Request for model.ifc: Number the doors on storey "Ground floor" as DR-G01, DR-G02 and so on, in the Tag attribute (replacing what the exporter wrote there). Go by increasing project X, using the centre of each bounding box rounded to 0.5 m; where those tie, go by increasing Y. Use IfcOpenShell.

First a look at what the model holds.

```python
import ifcopenshell
import ifcopenshell.util.element
import ifcopenshell.util.placement

model = ifcopenshell.open("model.ifc")
print(model.schema)
storey = next(s for s in model.by_type("IfcBuildingStorey") if s.Name == "Ground floor")
doors = [e for e in ifcopenshell.util.element.get_decomposition(storey) if e.is_a("IfcDoor")]
for e in sorted(doors, key=lambda e: e.id()):
    origin = ifcopenshell.util.placement.get_local_placement(e.ObjectPlacement)[:3, 3]
    print(e.id(), e.Tag, e.Name, origin.round(2) + 0.0, sep=" | ")
```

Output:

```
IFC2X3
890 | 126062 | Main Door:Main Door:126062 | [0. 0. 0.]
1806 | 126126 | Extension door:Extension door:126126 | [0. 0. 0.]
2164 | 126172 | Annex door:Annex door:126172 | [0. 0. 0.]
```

```python
import ifcopenshell
import ifcopenshell.geom
import ifcopenshell.util.element
import ifcopenshell.util.shape

model = ifcopenshell.open("model.ifc")
settings = ifcopenshell.geom.settings()
settings.set("use-world-coords", True)


def centre(element):
    shape = ifcopenshell.geom.create_shape(settings, element)
    return ifcopenshell.util.shape.get_bbox_centroid(shape.geometry)


storey = next(s for s in model.by_type("IfcBuildingStorey") if s.Name == "Ground floor")
doors = [e for e in ifcopenshell.util.element.get_decomposition(storey) if e.is_a("IfcDoor")]

# Insertion points can sit at a corner or the storey origin, so sort by the geometry (in metres).
centres = {e: centre(e) for e in doors}
doors.sort(key=lambda e: (round(centres[e][0] / 0.5), centres[e][1]))

for i, e in enumerate(doors, start=1):
    number = f"DR-G{i:02d}"
    e.Tag = number
    print(e.id(), number)

model.write("model_edited.ifc")
```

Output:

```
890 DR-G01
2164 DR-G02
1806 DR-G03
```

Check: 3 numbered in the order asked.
